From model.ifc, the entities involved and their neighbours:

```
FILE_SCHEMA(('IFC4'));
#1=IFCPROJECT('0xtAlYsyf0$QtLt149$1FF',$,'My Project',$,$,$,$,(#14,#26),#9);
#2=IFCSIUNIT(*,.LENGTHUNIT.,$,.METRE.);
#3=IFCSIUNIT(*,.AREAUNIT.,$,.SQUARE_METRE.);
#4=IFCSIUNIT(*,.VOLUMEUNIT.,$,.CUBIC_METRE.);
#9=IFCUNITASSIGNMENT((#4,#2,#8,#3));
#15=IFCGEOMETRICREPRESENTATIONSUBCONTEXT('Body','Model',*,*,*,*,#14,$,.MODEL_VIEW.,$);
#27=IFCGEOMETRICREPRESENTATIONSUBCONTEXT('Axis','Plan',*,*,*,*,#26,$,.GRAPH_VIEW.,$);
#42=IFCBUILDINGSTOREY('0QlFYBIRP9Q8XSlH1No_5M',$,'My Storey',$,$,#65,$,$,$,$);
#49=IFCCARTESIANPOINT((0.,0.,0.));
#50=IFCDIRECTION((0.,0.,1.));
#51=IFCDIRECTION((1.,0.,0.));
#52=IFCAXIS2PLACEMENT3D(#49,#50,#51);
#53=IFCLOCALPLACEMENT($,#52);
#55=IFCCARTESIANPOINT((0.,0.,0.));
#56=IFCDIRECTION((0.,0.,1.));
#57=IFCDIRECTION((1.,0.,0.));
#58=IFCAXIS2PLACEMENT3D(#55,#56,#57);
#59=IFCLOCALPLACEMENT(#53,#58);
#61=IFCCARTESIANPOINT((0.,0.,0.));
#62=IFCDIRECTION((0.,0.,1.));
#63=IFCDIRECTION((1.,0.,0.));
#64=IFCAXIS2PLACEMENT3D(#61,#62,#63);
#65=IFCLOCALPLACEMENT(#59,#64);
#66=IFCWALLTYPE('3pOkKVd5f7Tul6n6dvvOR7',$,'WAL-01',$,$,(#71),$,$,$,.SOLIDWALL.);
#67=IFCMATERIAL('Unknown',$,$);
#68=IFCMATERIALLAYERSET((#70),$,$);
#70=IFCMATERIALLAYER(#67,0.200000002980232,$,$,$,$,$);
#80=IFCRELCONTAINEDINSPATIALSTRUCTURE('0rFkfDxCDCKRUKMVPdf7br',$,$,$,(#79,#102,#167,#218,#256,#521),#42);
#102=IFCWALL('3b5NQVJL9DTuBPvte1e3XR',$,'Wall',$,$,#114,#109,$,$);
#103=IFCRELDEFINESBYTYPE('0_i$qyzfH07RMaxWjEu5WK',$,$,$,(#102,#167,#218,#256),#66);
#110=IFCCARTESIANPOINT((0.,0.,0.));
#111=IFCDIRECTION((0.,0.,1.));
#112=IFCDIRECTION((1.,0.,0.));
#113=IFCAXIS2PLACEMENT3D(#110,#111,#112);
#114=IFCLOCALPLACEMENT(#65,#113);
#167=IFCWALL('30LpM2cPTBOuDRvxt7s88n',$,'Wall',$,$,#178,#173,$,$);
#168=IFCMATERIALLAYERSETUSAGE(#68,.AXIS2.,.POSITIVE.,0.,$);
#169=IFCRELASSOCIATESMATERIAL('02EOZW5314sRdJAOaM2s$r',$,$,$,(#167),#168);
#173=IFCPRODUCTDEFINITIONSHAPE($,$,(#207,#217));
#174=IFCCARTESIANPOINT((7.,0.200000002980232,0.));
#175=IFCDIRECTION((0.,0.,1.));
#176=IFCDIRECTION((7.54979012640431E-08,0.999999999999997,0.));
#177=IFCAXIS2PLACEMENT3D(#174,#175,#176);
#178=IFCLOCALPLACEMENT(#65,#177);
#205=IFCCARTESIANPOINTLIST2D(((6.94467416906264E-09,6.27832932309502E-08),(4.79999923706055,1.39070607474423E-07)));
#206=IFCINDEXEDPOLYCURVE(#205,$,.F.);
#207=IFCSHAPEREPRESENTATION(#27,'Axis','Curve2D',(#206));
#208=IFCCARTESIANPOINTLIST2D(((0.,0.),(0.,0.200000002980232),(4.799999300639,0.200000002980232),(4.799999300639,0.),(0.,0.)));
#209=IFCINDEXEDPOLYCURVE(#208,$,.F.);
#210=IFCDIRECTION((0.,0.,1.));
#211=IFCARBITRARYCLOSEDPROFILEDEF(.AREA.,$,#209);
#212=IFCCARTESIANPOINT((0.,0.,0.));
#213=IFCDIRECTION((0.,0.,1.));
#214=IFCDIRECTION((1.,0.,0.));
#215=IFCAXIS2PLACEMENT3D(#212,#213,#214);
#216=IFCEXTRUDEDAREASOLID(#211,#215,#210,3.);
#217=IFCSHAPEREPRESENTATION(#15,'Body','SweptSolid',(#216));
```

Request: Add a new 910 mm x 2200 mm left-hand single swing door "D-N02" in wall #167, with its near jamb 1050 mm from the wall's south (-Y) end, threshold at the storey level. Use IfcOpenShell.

```python
import numpy as np
import ifcopenshell
import ifcopenshell.api.feature
import ifcopenshell.api.geometry
import ifcopenshell.api.root
import ifcopenshell.api.spatial
import ifcopenshell.geom
import ifcopenshell.util.element
import ifcopenshell.util.placement
import ifcopenshell.util.representation
import ifcopenshell.util.shape
import ifcopenshell.util.unit

model = ifcopenshell.open("model.ifc")
unit_scale = ifcopenshell.util.unit.calculate_unit_scale(model)
settings = ifcopenshell.geom.settings()


def volume(element):
    """Net volume in cubic metres, openings subtracted."""
    shape = ifcopenshell.geom.create_shape(settings, element)
    return ifcopenshell.util.shape.get_volume(shape.geometry)


wall = model.by_guid("30LpM2cPTBOuDRvxt7s88n")
storey = ifcopenshell.util.element.get_container(wall, ifc_class="IfcBuildingStorey")
context = ifcopenshell.util.representation.get_context(model, "Model", "Body", "MODEL_VIEW")
before = volume(wall)

width, height, from_end, sill = 0.91, 2.2, 1.05, 0.0  # metres

# The wall runs along its own X axis, and the end named is its -X end.
wall_shape = ifcopenshell.geom.create_shape(settings, wall)
x, y, z = ifcopenshell.util.shape.get_vertices(wall_shape.geometry).T
start = x.min() + from_end
face, thickness = float(y.min()), float(y.max() - y.min())
wall_matrix = ifcopenshell.util.placement.get_local_placement(wall.ObjectPlacement)
level = ifcopenshell.util.placement.get_local_placement(storey.ObjectPlacement)[2, 3]


def in_wall(x, y):
    """Placement at x, y metres in the wall's axes, at sill height."""
    matrix = wall_matrix.copy()
    matrix[:, 3] = wall_matrix @ np.array([x / unit_scale, y / unit_scale, 0.0, 1.0])
    matrix[2, 3] = level + sill / unit_scale
    return matrix


# Opening: a box that overshoots both wall faces by 50 mm.
opening = ifcopenshell.api.root.create_entity(model, ifc_class="IfcOpeningElement", predefined_type="OPENING")
box = ifcopenshell.api.geometry.add_wall_representation(
    model, context=context, length=width, height=height, thickness=thickness + 0.1
)
ifcopenshell.api.geometry.assign_representation(model, product=opening, representation=box)
ifcopenshell.api.geometry.edit_object_placement(model, product=opening, matrix=in_wall(start, face - 0.05), is_si=False)
ifcopenshell.api.feature.add_feature(model, feature=opening, element=wall)

door = ifcopenshell.api.root.create_entity(model, ifc_class="IfcDoor", name="D-N02", predefined_type="DOOR")
door.OverallWidth, door.OverallHeight = width / unit_scale, height / unit_scale
door.OperationType = "SINGLE_SWING_LEFT"
body = ifcopenshell.api.geometry.add_door_representation(
    model,
    context=context,
    overall_width=door.OverallWidth,
    overall_height=door.OverallHeight,
    operation_type="SINGLE_SWING_LEFT",
    lining_properties={"LiningDepth": thickness / unit_scale, "ThresholdDepth": thickness / unit_scale},
)
ifcopenshell.api.geometry.assign_representation(model, product=door, representation=body)
ifcopenshell.api.spatial.assign_container(model, products=[door], relating_structure=storey)
ifcopenshell.api.feature.add_filling(model, opening=opening, element=door)

# The lining spans the wall, so the door starts at the wall face.
ifcopenshell.api.geometry.edit_object_placement(model, product=door, matrix=in_wall(start, face), is_si=False)

after = volume(wall)

print(f"wall volume {before:.3f} -> {after:.3f} m3")

model.write("model_edited.ifc")
```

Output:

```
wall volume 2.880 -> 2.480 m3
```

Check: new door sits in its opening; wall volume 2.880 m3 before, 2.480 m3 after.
